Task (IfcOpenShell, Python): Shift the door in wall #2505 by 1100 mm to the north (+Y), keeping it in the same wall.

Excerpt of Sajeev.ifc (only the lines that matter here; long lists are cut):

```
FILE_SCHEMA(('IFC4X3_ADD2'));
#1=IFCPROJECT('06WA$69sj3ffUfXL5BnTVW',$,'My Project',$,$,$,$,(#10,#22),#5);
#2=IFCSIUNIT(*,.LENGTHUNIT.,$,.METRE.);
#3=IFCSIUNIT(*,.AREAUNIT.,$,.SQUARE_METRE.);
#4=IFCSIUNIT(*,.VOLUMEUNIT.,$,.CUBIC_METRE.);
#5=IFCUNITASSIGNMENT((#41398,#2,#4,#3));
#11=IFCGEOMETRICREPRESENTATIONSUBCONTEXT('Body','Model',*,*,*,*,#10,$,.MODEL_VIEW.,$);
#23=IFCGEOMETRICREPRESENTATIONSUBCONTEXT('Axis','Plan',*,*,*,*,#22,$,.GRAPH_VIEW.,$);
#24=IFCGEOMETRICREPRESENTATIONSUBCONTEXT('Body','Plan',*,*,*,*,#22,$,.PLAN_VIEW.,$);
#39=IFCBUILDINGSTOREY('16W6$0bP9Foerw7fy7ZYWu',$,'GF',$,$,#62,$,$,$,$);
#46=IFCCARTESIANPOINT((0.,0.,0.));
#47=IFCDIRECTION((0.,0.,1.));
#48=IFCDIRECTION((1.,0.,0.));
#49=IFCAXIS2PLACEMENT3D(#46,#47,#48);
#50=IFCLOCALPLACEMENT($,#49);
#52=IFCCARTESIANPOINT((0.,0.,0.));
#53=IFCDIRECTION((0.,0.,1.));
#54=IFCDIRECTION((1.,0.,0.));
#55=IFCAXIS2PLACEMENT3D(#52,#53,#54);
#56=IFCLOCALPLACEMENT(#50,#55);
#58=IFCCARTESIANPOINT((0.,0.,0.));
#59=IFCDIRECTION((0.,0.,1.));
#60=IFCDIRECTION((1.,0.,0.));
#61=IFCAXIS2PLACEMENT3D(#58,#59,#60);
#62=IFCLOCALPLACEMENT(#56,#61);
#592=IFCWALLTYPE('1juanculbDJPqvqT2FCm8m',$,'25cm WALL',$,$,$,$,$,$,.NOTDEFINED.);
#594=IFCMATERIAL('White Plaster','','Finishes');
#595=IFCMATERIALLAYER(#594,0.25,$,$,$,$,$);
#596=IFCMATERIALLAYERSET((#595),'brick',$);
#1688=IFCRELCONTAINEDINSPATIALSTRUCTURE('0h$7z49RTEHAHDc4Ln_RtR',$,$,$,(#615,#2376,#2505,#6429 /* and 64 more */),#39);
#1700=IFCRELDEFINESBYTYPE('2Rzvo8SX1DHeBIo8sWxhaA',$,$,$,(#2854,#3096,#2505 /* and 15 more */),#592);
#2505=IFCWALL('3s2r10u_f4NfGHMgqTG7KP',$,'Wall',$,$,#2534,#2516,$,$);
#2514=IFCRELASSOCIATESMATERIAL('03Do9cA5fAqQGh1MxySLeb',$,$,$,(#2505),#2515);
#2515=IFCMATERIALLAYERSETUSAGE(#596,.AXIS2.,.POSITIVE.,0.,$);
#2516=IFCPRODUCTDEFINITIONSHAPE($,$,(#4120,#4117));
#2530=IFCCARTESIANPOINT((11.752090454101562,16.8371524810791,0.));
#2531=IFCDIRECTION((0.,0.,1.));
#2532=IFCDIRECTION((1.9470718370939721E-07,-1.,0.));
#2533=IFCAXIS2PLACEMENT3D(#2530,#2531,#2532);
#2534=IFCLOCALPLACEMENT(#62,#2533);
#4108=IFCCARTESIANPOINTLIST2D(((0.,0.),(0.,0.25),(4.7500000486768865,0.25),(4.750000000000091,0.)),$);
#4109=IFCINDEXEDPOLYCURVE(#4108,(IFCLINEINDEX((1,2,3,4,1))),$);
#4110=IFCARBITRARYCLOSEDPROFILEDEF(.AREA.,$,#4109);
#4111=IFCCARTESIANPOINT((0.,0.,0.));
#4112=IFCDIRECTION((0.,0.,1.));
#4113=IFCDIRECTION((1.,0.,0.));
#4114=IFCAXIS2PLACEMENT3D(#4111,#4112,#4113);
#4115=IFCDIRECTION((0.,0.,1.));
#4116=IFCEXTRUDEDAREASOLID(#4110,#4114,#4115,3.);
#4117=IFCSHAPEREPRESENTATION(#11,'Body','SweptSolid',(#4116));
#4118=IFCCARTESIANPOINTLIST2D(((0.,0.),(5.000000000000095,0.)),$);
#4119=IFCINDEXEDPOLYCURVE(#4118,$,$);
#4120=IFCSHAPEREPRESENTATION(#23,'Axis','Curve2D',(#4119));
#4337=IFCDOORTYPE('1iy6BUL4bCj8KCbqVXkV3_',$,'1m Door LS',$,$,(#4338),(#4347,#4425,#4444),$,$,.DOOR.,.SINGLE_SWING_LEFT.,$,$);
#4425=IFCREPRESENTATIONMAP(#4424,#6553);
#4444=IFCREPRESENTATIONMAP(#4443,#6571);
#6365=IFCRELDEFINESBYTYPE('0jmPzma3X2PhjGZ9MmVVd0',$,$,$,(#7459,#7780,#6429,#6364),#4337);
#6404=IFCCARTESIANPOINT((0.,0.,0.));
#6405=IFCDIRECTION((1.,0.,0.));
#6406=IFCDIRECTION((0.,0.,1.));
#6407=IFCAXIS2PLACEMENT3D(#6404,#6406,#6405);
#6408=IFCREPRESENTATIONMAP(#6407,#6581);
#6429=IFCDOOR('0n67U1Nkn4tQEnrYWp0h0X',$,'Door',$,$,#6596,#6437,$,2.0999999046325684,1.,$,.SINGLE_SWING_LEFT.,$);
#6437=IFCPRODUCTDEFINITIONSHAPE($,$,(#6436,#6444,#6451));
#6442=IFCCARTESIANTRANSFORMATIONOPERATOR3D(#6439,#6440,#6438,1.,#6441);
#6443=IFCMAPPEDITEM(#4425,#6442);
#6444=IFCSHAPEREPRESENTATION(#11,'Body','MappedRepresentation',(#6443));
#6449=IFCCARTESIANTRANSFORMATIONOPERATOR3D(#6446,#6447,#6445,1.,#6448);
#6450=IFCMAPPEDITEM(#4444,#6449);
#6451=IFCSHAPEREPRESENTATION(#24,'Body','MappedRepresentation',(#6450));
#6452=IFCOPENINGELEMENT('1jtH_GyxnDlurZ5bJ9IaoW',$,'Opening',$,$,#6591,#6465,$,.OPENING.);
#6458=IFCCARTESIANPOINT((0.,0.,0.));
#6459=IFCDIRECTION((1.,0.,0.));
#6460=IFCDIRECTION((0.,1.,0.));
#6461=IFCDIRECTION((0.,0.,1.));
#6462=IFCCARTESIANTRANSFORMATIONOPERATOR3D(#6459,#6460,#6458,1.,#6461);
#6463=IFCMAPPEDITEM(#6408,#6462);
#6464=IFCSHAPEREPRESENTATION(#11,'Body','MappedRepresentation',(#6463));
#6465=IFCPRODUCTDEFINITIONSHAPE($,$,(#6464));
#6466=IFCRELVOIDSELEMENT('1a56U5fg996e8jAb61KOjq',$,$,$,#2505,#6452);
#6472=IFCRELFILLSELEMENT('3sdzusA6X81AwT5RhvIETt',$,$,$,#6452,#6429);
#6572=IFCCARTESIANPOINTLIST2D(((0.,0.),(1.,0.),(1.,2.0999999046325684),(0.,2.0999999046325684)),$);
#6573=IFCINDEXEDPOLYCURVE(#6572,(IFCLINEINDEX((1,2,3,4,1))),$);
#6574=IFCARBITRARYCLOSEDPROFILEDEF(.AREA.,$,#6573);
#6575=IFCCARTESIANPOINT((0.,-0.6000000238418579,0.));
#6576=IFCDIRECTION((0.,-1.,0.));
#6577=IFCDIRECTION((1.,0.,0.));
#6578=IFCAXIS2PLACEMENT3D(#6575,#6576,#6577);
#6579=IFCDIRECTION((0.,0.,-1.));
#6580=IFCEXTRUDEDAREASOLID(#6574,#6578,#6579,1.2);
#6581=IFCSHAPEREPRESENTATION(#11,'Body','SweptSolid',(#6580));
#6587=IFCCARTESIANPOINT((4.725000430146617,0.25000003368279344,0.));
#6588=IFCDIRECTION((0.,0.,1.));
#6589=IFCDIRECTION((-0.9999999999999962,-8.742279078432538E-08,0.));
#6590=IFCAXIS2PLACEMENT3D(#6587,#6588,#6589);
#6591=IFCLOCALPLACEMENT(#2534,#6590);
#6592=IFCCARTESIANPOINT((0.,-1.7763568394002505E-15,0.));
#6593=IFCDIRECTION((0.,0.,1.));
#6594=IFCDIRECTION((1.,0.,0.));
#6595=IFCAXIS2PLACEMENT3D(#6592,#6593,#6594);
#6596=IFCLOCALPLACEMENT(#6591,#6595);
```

```python
import ifcopenshell
import ifcopenshell.api.geometry
import ifcopenshell.util.placement
import ifcopenshell.util.unit

model = ifcopenshell.open("Sajeev.ifc")
unit_scale = ifcopenshell.util.unit.calculate_unit_scale(model)

door = model.by_id(6429)
opening = door.FillsVoids[0].RelatingOpeningElement
wall = opening.VoidsElements[0].RelatingBuildingElement

wall_matrix = ifcopenshell.util.placement.get_local_placement(wall.ObjectPlacement)
shift = wall_matrix[:3, 0] * -1.1 / unit_scale
before = ifcopenshell.util.placement.get_local_placement(door.ObjectPlacement)[:3, 3].copy()

# The door is placed relative to its opening, so it follows when the opening moves.
matrix = ifcopenshell.util.placement.get_local_placement(opening.ObjectPlacement)
matrix[:3, 3] += shift
ifcopenshell.api.geometry.edit_object_placement(
    model, product=opening, matrix=matrix, is_si=False, should_transform_children=True
)

after = ifcopenshell.util.placement.get_local_placement(door.ObjectPlacement)[:3, 3]
print("door moved by", (after - before).round(3) + 0.0)

model.write("Sajeev_rev.ifc")
```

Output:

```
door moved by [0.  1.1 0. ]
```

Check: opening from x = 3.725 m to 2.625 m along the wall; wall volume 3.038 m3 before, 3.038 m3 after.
